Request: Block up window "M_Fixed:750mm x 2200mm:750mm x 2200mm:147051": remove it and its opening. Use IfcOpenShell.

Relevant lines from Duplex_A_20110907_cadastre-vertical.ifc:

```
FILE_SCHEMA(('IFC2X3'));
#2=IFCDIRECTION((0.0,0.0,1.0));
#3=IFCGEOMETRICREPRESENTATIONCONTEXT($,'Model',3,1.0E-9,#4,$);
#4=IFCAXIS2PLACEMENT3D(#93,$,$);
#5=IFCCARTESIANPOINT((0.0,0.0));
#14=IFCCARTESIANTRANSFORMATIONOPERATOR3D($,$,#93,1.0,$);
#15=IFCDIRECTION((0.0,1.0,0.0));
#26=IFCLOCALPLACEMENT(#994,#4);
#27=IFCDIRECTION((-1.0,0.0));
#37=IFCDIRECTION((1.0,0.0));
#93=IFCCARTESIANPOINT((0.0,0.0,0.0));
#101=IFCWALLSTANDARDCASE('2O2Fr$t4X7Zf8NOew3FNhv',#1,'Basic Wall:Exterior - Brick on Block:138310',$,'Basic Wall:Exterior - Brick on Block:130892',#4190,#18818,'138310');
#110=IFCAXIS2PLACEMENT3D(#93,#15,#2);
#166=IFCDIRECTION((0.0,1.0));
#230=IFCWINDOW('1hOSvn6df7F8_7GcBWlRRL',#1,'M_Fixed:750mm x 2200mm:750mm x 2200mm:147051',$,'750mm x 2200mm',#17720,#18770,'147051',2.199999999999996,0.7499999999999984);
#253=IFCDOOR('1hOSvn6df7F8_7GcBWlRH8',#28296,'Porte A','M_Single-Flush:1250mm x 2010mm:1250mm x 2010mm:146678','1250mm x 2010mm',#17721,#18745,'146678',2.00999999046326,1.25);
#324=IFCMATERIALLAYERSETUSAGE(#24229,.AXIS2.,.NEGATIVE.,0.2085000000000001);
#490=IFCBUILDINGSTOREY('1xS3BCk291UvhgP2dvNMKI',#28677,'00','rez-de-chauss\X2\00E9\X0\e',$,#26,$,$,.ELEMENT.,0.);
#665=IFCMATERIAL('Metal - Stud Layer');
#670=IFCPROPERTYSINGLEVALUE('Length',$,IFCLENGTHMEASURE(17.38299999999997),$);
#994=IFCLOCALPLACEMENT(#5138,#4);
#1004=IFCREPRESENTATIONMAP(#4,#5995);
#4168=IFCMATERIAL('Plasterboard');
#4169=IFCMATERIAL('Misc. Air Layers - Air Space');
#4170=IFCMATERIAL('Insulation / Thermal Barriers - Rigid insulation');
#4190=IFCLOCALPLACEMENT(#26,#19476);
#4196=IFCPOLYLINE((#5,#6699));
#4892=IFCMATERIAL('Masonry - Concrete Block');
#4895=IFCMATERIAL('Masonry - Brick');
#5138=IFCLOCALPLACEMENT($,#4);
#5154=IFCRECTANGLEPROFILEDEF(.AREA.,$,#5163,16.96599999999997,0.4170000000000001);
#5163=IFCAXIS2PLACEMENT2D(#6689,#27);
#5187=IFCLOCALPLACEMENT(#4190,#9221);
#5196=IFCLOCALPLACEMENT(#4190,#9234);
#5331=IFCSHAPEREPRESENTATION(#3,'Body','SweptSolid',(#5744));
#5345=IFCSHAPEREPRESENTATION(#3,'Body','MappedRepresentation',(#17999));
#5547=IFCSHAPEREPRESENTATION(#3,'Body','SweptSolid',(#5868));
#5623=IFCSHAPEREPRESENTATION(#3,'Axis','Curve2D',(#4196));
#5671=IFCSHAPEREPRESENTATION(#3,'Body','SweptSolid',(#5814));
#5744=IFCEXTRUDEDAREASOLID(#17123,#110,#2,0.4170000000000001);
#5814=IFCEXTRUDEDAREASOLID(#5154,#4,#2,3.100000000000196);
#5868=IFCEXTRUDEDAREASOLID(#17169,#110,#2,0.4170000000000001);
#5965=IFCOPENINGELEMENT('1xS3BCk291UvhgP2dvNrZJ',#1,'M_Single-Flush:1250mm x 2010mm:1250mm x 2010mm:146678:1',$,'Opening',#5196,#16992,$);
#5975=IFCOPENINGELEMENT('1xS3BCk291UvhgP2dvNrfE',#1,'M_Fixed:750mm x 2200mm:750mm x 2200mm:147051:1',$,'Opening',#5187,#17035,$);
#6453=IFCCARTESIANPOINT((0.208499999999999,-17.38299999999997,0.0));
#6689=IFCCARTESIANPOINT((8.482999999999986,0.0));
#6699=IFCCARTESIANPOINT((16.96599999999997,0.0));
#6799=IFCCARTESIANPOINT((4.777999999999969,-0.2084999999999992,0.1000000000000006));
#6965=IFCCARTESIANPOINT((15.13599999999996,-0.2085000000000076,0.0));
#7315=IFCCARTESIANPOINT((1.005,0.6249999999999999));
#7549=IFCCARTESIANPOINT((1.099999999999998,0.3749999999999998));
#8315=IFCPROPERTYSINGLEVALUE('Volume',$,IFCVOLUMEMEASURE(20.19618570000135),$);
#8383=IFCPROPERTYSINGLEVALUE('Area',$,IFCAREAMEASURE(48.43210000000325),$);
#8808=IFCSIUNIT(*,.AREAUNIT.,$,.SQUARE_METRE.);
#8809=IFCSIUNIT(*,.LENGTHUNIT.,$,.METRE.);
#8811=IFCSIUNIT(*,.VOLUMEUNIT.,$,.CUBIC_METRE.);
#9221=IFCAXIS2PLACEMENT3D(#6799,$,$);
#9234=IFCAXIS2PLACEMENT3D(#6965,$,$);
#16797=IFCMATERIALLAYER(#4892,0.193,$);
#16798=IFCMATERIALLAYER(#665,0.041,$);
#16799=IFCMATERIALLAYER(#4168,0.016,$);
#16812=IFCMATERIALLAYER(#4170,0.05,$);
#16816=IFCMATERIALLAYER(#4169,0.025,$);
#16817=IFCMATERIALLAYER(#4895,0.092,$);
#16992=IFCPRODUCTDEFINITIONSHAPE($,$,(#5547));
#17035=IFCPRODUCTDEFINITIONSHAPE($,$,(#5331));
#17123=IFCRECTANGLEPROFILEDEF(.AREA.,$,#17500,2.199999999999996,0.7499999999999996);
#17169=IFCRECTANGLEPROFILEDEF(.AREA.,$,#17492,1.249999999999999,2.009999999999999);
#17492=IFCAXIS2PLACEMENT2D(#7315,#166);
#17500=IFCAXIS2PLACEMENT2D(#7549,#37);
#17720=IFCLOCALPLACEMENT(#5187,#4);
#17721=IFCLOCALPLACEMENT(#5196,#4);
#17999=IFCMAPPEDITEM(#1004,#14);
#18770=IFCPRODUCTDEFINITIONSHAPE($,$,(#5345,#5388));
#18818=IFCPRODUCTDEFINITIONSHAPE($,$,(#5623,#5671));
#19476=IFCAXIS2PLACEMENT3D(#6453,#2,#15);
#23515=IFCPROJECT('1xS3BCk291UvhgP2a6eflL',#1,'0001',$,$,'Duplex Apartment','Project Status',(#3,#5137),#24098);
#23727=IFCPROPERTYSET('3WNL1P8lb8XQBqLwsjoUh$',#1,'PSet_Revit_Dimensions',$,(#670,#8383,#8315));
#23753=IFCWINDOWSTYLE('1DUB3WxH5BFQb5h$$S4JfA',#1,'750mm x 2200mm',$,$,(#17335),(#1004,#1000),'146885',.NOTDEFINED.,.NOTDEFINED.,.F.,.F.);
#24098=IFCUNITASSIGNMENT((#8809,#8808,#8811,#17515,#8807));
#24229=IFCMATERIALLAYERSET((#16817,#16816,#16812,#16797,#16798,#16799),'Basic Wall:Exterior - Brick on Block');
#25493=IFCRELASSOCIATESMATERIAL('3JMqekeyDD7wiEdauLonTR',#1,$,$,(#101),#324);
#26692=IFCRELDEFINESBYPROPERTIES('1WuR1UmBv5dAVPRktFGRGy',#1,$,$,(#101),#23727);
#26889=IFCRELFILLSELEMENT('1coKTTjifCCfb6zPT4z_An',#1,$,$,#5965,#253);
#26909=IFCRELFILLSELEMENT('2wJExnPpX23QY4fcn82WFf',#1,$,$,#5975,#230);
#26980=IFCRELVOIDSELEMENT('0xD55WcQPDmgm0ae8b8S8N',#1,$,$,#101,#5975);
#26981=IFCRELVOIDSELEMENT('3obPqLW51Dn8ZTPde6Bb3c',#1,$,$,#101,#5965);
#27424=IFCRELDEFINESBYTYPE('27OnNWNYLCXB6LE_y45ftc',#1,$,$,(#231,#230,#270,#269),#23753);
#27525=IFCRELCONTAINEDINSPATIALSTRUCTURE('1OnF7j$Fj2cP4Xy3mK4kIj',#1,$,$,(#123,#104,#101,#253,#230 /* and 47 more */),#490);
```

```python
import ifcopenshell
import ifcopenshell.api.feature
import ifcopenshell.api.pset
import ifcopenshell.api.root
import ifcopenshell.geom
import ifcopenshell.util.element
import ifcopenshell.util.shape
import ifcopenshell.util.unit

model = ifcopenshell.open("Duplex_A_20110907_cadastre-vertical.ifc")
area_scale = ifcopenshell.util.unit.calculate_unit_scale(model, "AREAUNIT")
volume_scale = ifcopenshell.util.unit.calculate_unit_scale(model, "VOLUMEUNIT")
settings = ifcopenshell.geom.settings()


def volume(element):
    """Net volume in cubic metres, openings subtracted."""
    shape = ifcopenshell.geom.create_shape(settings, element)
    return ifcopenshell.util.shape.get_volume(shape.geometry)


window = model.by_guid("1hOSvn6df7F8_7GcBWlRRL")
opening = window.FillsVoids[0].RelatingOpeningElement
wall = opening.VoidsElements[0].RelatingBuildingElement
before = volume(wall)

ifcopenshell.api.root.remove_product(model, product=window)
ifcopenshell.api.feature.remove_feature(model, feature=opening)

after = volume(wall)
thickness = 0.417  # wall thickness in metres

# Update the wall's stored quantities.
pset = model.by_id(ifcopenshell.util.element.get_pset(wall, "PSet_Revit_Dimensions", should_inherit=False)["id"])
ifcopenshell.api.pset.edit_pset(model, pset=pset, properties={
    "Area": model.create_entity("IfcAreaMeasure", after / thickness / area_scale),
    "Volume": model.create_entity("IfcVolumeMeasure", after / volume_scale),
})

print(f"wall volume {before:.3f} -> {after:.3f} m3")

model.write("Duplex_A_20110907_cadastre-vertical_rev.ifc")
```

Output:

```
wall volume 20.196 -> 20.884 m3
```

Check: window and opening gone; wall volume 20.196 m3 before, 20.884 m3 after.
